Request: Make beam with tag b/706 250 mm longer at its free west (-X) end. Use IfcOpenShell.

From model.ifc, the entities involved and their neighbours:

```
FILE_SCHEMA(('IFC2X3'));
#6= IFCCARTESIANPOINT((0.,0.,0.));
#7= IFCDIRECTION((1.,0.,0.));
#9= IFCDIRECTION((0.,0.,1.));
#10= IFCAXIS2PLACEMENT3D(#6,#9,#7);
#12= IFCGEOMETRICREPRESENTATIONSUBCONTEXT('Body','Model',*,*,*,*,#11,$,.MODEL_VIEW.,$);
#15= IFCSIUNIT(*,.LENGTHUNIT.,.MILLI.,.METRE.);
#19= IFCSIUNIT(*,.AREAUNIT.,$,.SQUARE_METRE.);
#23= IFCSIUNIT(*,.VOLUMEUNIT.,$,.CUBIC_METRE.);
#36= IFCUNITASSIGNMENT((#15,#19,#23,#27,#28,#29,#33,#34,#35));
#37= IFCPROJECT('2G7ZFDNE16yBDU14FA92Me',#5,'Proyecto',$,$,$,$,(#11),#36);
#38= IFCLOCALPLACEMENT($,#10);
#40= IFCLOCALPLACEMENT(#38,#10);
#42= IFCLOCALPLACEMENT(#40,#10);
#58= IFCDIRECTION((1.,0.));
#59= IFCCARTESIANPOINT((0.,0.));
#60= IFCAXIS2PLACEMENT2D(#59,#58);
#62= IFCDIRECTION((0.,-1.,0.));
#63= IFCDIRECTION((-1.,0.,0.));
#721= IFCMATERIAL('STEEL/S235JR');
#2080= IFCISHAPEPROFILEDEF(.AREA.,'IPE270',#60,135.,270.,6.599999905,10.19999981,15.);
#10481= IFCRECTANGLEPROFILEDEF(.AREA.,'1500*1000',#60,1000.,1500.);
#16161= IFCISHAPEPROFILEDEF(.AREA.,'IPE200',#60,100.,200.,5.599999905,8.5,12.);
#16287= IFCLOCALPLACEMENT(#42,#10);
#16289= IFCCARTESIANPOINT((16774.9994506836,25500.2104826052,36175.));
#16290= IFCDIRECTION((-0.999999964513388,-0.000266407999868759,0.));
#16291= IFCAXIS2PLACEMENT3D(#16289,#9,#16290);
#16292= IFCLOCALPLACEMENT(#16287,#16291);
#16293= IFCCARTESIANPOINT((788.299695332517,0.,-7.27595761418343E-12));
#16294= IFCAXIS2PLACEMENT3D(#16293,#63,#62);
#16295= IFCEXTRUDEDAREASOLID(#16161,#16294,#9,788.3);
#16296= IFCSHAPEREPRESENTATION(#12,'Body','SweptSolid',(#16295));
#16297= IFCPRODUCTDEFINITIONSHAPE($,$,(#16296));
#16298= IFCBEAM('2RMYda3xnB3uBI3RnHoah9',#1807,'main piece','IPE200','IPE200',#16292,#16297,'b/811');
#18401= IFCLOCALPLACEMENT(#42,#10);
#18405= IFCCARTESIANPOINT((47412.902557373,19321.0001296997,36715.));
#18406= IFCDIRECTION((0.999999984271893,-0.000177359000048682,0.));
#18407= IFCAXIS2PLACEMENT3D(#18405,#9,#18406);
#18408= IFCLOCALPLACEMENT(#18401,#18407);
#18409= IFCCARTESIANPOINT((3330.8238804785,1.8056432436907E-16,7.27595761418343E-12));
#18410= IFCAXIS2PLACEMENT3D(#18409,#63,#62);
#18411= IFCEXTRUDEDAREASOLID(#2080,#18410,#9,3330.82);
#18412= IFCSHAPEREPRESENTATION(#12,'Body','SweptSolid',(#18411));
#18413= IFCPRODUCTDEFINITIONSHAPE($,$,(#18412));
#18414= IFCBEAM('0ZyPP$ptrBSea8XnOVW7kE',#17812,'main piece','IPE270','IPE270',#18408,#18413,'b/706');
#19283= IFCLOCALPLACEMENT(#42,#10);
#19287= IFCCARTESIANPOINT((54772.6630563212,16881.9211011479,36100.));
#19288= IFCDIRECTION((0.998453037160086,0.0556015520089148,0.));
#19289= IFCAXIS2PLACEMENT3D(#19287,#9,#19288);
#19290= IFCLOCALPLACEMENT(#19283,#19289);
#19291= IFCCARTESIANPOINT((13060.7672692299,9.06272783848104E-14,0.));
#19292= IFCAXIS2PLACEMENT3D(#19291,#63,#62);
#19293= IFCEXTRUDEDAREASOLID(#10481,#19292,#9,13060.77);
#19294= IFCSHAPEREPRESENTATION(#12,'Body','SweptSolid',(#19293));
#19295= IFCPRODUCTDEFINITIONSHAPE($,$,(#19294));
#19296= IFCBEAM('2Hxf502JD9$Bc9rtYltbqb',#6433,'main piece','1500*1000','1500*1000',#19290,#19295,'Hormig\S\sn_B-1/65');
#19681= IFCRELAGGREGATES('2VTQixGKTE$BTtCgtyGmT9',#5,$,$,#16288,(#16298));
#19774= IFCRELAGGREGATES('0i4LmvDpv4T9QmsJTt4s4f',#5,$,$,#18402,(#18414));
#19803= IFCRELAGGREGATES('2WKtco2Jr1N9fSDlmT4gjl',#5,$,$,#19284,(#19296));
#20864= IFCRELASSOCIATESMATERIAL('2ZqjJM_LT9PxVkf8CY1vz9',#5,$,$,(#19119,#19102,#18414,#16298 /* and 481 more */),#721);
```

```python
import ifcopenshell
import ifcopenshell.util.representation

model = ifcopenshell.open("model.ifc")

member = model.by_guid("0ZyPP$ptrBSea8XnOVW7kE")
change = 250.0

# The extrusion runs towards the end named, so only its depth changes.
body = ifcopenshell.util.representation.get_representation(member, "Model", "Body")
solid = body.Items[0]
old_length = solid.Depth
solid.Depth += change

print(f"length {old_length:g} -> {solid.Depth:g}")

model.write("model_updated.ifc")
```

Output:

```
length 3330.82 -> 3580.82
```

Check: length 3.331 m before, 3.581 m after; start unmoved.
